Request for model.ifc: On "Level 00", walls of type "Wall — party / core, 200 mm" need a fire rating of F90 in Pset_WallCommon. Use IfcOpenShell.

First a look at what the model holds.

```python
import ifcopenshell
import ifcopenshell.util.element

model = ifcopenshell.open("model.ifc")
print(model.schema)
storey = next(s for s in model.by_type("IfcBuildingStorey") if s.Name == "Level 00")
walls = [e for e in ifcopenshell.util.element.get_decomposition(storey) if e.is_a("IfcWall")]
seen = {}
for e in walls:
    element_type = ifcopenshell.util.element.get_type(e)
    key = (element_type.Name if element_type != e and element_type else None, ifcopenshell.util.element.get_pset(e, "Pset_WallCommon", "FireRating"))
    seen[key] = seen.get(key, 0) + 1
for (name, value), count in sorted(seen.items(), key=str):
    print(count, "x", name, "|", value)
```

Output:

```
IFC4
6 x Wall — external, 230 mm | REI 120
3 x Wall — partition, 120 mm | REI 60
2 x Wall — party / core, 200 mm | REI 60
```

```python
import ifcopenshell
import ifcopenshell.api.pset
import ifcopenshell.util.element

model = ifcopenshell.open("model.ifc")

storey = next(s for s in model.by_type("IfcBuildingStorey") if s.Name == "Level 00")
walls = [e for e in ifcopenshell.util.element.get_decomposition(storey) if e.is_a("IfcWall")]

count = 0
for e in walls:
    element_type = ifcopenshell.util.element.get_type(e)
    if element_type in (None, e) or element_type.Name != "Wall — party / core, 200 mm":
        continue
    # add_pset returns the element's existing set when there is one.
    pset = ifcopenshell.api.pset.add_pset(model, product=e, name="Pset_WallCommon")
    ifcopenshell.api.pset.edit_pset(model, pset=pset, properties={"FireRating": "F90"})
    count += 1

print(count, "walls updated")

model.write("model_updated.ifc")
```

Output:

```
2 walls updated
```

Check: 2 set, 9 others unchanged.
